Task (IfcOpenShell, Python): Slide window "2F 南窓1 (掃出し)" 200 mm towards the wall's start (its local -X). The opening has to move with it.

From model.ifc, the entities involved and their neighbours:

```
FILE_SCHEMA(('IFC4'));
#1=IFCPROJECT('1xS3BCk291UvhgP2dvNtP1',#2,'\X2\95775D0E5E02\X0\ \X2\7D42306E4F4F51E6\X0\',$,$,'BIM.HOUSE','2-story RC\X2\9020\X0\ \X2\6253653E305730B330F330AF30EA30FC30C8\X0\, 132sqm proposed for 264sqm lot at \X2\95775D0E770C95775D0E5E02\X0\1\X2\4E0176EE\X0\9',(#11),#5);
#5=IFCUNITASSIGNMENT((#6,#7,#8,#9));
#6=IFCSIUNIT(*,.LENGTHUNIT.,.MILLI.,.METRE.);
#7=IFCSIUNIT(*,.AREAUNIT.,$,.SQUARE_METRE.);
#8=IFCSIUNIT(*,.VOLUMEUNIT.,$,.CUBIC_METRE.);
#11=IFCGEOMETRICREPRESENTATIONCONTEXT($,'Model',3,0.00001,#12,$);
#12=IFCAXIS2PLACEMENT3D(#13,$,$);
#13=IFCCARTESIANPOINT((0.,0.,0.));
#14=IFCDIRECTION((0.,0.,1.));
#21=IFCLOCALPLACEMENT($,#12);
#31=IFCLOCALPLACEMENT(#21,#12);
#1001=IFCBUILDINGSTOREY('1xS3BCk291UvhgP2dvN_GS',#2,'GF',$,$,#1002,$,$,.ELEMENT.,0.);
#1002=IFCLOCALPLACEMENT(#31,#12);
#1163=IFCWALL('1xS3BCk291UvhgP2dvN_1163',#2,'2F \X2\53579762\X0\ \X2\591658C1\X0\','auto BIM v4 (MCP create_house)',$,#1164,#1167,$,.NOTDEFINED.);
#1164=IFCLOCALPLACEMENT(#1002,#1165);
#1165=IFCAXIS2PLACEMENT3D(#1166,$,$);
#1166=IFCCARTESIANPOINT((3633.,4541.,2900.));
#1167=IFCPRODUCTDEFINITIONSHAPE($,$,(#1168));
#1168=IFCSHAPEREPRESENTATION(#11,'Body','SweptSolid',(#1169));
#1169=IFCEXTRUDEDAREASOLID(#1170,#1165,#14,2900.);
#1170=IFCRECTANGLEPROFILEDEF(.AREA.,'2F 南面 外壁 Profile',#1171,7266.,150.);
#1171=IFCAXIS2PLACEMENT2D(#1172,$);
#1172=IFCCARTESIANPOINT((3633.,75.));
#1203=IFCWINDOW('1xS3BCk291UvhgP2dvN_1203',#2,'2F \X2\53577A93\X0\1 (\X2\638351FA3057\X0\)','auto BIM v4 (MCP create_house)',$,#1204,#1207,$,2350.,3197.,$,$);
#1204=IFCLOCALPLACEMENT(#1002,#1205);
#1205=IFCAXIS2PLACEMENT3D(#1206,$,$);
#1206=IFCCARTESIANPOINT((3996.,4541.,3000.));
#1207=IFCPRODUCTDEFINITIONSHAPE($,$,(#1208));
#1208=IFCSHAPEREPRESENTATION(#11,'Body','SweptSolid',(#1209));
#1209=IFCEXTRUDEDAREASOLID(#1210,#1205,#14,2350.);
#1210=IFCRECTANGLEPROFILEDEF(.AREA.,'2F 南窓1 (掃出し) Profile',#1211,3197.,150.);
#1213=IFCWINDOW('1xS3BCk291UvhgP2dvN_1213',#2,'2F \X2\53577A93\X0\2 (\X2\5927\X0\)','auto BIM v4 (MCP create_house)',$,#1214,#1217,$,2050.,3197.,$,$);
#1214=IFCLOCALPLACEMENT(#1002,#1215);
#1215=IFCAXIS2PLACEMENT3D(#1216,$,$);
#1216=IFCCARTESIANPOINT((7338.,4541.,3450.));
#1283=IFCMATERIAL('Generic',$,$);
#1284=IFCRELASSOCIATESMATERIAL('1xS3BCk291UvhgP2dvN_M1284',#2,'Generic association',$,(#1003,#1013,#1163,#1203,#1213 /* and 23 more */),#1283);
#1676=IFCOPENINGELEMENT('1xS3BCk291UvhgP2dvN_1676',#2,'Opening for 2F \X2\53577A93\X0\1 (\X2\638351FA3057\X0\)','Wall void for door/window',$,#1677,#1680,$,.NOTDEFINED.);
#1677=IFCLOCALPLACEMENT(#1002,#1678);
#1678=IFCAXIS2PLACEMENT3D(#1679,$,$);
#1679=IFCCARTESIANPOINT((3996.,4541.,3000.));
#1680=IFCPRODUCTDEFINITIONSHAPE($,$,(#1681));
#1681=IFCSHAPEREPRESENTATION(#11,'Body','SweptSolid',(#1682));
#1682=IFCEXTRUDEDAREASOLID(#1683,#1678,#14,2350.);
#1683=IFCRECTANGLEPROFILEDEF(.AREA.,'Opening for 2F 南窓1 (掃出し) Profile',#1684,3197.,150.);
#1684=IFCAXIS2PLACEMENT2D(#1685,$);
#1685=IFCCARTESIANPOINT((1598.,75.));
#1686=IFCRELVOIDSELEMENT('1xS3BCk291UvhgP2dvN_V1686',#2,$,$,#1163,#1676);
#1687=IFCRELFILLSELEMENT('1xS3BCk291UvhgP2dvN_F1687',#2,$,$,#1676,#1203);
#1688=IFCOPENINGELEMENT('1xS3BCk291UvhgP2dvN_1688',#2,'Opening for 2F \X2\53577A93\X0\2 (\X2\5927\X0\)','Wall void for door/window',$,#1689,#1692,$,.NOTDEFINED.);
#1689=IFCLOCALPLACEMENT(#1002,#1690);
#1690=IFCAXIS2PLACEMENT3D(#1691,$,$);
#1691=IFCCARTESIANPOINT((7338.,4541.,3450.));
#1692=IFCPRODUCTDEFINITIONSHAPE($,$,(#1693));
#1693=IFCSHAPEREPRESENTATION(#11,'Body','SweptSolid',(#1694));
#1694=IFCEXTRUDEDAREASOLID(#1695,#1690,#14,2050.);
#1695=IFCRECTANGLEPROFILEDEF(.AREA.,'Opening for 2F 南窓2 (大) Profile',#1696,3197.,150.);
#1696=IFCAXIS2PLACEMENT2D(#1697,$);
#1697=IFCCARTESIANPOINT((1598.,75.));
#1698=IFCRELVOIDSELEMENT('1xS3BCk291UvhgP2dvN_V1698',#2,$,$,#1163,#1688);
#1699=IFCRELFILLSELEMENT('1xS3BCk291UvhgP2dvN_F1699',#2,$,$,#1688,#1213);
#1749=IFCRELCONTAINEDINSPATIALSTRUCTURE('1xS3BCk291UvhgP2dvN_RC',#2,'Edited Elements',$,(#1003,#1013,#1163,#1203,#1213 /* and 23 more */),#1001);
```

```python
import ifcopenshell
import ifcopenshell.api.geometry
import ifcopenshell.util.placement
import ifcopenshell.util.unit

model = ifcopenshell.open("model.ifc")
unit_scale = ifcopenshell.util.unit.calculate_unit_scale(model)

window = model.by_guid("1xS3BCk291UvhgP2dvN_1203")
opening = window.FillsVoids[0].RelatingOpeningElement
wall = opening.VoidsElements[0].RelatingBuildingElement

wall_matrix = ifcopenshell.util.placement.get_local_placement(wall.ObjectPlacement)
shift = wall_matrix[:3, 0] * -0.2 / unit_scale
before = ifcopenshell.util.placement.get_local_placement(window.ObjectPlacement)[:3, 3].copy()

# The window is not placed relative to its opening, so move both.
for product in (opening, window):
    matrix = ifcopenshell.util.placement.get_local_placement(product.ObjectPlacement)
    matrix[:3, 3] += shift
    ifcopenshell.api.geometry.edit_object_placement(model, product=product, matrix=matrix, is_si=False)

after = ifcopenshell.util.placement.get_local_placement(window.ObjectPlacement)[:3, 3]
print("window moved by", (after - before).round(3) + 0.0)

model.write("model_updated.ifc")
```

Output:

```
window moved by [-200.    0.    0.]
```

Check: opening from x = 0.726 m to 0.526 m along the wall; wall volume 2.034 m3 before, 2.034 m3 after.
